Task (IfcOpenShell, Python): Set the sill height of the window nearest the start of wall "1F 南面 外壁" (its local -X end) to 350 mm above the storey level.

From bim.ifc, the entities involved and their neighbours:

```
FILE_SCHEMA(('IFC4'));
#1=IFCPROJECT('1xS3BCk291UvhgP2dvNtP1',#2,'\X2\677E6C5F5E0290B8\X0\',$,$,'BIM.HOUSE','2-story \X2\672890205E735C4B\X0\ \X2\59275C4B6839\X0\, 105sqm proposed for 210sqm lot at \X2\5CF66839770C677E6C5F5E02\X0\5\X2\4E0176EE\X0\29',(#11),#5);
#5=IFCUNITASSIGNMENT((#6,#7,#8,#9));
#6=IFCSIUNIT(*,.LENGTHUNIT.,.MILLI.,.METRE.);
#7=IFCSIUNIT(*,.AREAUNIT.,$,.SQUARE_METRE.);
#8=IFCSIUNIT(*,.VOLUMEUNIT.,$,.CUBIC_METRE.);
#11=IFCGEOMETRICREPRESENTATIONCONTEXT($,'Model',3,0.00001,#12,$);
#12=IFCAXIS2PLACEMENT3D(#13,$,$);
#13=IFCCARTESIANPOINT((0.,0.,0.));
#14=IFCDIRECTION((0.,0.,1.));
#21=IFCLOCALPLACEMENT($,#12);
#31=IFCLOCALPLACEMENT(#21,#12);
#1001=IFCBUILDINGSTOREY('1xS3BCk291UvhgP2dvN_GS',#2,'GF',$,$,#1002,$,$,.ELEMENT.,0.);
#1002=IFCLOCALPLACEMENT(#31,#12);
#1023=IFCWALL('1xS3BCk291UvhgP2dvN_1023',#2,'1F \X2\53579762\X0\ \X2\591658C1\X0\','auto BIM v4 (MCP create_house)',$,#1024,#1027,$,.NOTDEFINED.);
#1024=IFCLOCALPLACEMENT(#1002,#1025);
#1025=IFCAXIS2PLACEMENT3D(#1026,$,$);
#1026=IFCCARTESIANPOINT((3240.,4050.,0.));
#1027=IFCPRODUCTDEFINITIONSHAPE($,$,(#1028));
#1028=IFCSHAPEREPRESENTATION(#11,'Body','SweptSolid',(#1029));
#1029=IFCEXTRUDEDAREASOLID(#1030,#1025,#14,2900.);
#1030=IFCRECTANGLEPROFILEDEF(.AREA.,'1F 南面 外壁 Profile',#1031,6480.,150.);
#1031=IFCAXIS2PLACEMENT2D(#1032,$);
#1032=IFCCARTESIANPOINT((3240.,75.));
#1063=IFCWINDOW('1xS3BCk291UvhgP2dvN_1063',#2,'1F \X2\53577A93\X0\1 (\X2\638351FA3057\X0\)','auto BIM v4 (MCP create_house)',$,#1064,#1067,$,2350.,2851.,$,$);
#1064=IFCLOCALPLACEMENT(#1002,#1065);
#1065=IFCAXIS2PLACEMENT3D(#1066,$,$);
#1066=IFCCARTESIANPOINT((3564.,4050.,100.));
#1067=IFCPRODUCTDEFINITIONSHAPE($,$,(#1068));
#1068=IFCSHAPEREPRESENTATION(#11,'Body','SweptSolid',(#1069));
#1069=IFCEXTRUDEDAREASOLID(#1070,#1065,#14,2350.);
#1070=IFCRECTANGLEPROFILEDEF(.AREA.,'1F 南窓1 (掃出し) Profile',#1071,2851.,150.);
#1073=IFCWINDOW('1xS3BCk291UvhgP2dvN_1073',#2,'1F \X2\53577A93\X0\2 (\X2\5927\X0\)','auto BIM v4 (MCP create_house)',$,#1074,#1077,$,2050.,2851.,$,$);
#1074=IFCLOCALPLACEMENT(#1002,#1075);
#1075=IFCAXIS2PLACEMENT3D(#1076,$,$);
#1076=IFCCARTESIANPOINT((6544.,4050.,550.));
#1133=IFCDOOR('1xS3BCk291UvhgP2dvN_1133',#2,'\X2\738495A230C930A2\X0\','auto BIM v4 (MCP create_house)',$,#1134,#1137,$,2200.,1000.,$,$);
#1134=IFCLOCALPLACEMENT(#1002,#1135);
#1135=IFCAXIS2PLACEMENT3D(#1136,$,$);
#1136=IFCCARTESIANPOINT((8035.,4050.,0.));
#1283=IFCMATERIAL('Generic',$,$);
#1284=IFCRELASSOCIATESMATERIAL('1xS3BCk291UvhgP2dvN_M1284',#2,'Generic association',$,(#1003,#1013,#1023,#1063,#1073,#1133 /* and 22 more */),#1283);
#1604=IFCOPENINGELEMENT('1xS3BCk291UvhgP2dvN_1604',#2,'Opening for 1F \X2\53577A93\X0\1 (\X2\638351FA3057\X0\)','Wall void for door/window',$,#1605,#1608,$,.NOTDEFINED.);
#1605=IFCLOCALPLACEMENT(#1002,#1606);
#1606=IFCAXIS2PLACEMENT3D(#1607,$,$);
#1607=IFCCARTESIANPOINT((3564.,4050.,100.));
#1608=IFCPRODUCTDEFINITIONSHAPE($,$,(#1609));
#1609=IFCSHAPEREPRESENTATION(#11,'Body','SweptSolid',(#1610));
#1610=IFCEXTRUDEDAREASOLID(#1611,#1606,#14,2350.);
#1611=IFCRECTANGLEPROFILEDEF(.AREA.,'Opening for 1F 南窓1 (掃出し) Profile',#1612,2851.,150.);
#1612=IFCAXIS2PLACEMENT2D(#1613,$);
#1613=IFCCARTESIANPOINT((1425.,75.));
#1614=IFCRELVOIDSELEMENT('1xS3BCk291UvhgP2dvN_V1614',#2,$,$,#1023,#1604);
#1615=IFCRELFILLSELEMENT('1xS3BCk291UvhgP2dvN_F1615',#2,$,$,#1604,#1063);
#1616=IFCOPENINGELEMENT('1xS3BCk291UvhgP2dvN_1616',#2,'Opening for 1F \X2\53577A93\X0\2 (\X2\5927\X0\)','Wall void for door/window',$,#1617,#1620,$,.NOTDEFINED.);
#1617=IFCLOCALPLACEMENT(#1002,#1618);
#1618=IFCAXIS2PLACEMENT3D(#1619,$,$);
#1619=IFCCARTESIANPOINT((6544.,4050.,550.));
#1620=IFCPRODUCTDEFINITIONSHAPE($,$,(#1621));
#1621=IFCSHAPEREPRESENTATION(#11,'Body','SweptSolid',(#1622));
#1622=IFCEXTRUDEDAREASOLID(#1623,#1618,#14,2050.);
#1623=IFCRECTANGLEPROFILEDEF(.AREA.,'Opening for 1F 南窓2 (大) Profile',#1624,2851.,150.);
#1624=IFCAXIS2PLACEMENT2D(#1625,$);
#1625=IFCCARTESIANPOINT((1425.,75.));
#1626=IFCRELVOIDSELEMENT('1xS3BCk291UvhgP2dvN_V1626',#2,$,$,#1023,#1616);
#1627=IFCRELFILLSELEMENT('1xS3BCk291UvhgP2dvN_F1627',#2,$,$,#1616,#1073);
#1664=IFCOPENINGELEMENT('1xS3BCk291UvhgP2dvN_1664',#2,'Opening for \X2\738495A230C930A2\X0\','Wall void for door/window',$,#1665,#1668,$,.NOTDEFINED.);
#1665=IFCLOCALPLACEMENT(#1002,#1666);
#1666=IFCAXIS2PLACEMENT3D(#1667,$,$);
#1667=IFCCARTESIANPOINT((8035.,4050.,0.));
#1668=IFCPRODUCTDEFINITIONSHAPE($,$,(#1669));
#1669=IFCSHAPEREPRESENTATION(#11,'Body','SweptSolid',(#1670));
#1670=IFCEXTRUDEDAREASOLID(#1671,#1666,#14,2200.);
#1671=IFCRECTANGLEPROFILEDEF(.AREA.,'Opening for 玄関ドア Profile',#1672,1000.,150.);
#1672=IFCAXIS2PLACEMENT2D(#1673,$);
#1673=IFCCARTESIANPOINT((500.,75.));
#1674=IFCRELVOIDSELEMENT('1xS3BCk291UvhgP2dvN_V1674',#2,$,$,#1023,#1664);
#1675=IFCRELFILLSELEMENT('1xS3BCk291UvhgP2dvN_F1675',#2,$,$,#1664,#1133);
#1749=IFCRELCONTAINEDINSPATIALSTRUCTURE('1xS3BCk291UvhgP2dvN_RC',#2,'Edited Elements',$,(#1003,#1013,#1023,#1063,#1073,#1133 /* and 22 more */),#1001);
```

```python
import numpy as np
import ifcopenshell
import ifcopenshell.api.geometry
import ifcopenshell.geom
import ifcopenshell.util.element
import ifcopenshell.util.placement
import ifcopenshell.util.shape
import ifcopenshell.util.unit

model = ifcopenshell.open("bim.ifc")
unit_scale = ifcopenshell.util.unit.calculate_unit_scale(model)

window = model.by_guid("1xS3BCk291UvhgP2dvN_1063")
opening = window.FillsVoids[0].RelatingOpeningElement
storey = ifcopenshell.util.element.get_container(window, ifc_class="IfcBuildingStorey")
level = ifcopenshell.util.placement.get_local_placement(storey.ObjectPlacement)[2, 3]

# The opening's origin need not be at the sill, so measure its lowest point.
shape = ifcopenshell.geom.create_shape(ifcopenshell.geom.settings(), opening)
bottom = ifcopenshell.util.shape.get_shape_bottom_elevation(shape, shape.geometry) / unit_scale
dz = level + 0.35 / unit_scale - bottom

shift = np.array([0.0, 0.0, dz])
# The window is not placed relative to its opening, so move both.
for product in (opening, window):
    matrix = ifcopenshell.util.placement.get_local_placement(product.ObjectPlacement)
    matrix[:3, 3] += shift
    ifcopenshell.api.geometry.edit_object_placement(model, product=product, matrix=matrix, is_si=False)

print(f"moved by {dz * unit_scale:+.3f} m")

model.write("bim_edited.ifc")
```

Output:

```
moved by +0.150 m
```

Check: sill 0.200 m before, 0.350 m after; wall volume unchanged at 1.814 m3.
